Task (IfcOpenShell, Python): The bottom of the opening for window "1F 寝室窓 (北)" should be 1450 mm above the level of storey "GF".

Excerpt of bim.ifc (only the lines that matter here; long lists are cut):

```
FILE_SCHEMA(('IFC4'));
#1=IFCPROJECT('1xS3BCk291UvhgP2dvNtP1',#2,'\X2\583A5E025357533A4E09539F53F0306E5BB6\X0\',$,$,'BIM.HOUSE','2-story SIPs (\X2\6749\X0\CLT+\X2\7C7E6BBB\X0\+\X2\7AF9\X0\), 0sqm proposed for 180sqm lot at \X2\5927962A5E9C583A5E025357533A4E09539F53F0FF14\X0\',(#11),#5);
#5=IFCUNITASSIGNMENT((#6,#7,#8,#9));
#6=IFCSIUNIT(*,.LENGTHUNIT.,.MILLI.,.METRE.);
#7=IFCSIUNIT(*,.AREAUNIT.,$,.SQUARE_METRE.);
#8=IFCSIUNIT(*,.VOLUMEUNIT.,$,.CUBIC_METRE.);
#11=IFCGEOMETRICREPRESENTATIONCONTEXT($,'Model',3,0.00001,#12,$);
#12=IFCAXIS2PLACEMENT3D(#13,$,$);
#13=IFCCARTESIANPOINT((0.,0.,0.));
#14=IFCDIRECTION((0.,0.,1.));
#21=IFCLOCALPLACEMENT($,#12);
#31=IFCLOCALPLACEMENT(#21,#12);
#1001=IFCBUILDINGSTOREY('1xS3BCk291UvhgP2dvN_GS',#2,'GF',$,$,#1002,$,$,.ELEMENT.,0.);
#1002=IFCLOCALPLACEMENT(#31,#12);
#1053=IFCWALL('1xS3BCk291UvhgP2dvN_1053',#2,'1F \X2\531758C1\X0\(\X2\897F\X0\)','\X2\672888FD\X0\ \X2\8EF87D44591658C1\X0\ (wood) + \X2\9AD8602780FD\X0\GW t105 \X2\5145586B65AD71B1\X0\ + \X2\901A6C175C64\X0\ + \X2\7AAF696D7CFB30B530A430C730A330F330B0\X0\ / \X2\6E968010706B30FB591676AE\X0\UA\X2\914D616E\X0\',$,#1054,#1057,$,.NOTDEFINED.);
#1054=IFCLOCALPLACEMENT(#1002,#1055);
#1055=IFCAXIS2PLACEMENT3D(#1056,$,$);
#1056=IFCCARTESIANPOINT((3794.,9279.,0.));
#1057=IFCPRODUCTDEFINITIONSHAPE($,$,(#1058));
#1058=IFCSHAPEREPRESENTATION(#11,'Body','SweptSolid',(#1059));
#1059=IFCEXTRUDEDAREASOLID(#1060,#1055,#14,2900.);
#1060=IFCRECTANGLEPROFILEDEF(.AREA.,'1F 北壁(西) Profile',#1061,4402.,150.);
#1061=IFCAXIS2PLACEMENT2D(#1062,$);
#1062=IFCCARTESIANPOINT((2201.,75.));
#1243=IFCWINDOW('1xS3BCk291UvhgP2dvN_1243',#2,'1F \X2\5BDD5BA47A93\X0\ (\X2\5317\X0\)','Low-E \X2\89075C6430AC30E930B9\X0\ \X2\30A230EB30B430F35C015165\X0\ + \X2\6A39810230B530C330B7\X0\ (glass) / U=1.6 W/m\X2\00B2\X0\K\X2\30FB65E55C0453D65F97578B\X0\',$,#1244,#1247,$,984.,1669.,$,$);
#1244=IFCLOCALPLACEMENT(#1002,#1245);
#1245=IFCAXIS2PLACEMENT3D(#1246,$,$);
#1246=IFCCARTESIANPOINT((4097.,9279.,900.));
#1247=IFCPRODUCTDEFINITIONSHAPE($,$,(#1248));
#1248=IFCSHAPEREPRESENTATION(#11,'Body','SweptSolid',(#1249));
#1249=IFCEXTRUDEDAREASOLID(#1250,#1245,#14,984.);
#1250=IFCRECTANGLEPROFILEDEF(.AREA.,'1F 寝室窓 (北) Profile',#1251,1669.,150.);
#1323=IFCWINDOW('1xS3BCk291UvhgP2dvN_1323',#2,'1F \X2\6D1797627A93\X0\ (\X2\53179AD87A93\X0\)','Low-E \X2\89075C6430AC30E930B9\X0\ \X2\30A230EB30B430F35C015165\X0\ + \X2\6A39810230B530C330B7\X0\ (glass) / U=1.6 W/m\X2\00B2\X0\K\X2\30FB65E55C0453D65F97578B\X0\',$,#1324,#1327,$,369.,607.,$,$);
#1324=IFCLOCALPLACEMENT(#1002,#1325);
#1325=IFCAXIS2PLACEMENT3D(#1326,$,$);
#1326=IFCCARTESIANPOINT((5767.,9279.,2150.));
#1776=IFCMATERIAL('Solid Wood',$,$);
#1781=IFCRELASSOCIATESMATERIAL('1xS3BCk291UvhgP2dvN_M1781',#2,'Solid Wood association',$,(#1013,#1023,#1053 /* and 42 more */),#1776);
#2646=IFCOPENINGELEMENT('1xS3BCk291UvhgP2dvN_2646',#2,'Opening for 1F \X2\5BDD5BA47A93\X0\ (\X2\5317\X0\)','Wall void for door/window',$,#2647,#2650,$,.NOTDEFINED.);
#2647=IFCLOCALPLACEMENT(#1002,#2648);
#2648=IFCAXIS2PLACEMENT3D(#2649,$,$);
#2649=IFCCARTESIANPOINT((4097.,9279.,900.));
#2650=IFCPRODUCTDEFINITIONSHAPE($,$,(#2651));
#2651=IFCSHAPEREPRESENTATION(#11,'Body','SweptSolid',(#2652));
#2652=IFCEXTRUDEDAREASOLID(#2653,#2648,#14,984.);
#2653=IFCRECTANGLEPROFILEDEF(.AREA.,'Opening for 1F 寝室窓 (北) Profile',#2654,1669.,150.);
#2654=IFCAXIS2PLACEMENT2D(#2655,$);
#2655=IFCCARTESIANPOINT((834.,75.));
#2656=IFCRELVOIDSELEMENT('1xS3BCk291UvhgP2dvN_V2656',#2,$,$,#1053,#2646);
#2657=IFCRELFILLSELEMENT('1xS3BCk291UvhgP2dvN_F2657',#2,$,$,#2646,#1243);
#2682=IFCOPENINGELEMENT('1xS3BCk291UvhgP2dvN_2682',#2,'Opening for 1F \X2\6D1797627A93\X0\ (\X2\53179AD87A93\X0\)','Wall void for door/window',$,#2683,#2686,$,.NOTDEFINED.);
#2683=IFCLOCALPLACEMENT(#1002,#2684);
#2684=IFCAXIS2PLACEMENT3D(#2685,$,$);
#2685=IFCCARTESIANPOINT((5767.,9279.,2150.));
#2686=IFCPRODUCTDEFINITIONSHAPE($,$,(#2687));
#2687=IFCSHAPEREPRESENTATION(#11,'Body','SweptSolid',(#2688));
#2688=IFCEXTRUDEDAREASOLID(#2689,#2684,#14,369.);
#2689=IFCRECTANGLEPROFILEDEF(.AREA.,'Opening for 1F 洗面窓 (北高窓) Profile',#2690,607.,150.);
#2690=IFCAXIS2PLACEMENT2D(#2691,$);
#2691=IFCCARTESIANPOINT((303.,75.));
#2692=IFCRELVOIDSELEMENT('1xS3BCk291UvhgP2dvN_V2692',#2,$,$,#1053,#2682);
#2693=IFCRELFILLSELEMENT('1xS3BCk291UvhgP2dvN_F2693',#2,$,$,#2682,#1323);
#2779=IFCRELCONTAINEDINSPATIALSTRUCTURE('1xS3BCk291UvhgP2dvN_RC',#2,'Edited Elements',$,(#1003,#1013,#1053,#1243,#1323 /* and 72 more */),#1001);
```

```python
import numpy as np
import ifcopenshell
import ifcopenshell.api.geometry
import ifcopenshell.geom
import ifcopenshell.util.element
import ifcopenshell.util.placement
import ifcopenshell.util.shape
import ifcopenshell.util.unit

model = ifcopenshell.open("bim.ifc")
unit_scale = ifcopenshell.util.unit.calculate_unit_scale(model)

window = model.by_guid("1xS3BCk291UvhgP2dvN_1243")
opening = window.FillsVoids[0].RelatingOpeningElement
storey = ifcopenshell.util.element.get_container(window, ifc_class="IfcBuildingStorey")
level = ifcopenshell.util.placement.get_local_placement(storey.ObjectPlacement)[2, 3]

# The opening's origin need not be at the sill, so measure its lowest point.
shape = ifcopenshell.geom.create_shape(ifcopenshell.geom.settings(), opening)
bottom = ifcopenshell.util.shape.get_shape_bottom_elevation(shape, shape.geometry) / unit_scale
dz = level + 1450.0 - bottom

shift = np.array([0.0, 0.0, dz])
# The window is not placed relative to its opening, so move both.
for product in (opening, window):
    matrix = ifcopenshell.util.placement.get_local_placement(product.ObjectPlacement)
    matrix[:3, 3] += shift
    ifcopenshell.api.geometry.edit_object_placement(model, product=product, matrix=matrix, is_si=False)

print(f"moved by {dz * unit_scale:+.3f} m")

model.write("bim-out.ifc")
```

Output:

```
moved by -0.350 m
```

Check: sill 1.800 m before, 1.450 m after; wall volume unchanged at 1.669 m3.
